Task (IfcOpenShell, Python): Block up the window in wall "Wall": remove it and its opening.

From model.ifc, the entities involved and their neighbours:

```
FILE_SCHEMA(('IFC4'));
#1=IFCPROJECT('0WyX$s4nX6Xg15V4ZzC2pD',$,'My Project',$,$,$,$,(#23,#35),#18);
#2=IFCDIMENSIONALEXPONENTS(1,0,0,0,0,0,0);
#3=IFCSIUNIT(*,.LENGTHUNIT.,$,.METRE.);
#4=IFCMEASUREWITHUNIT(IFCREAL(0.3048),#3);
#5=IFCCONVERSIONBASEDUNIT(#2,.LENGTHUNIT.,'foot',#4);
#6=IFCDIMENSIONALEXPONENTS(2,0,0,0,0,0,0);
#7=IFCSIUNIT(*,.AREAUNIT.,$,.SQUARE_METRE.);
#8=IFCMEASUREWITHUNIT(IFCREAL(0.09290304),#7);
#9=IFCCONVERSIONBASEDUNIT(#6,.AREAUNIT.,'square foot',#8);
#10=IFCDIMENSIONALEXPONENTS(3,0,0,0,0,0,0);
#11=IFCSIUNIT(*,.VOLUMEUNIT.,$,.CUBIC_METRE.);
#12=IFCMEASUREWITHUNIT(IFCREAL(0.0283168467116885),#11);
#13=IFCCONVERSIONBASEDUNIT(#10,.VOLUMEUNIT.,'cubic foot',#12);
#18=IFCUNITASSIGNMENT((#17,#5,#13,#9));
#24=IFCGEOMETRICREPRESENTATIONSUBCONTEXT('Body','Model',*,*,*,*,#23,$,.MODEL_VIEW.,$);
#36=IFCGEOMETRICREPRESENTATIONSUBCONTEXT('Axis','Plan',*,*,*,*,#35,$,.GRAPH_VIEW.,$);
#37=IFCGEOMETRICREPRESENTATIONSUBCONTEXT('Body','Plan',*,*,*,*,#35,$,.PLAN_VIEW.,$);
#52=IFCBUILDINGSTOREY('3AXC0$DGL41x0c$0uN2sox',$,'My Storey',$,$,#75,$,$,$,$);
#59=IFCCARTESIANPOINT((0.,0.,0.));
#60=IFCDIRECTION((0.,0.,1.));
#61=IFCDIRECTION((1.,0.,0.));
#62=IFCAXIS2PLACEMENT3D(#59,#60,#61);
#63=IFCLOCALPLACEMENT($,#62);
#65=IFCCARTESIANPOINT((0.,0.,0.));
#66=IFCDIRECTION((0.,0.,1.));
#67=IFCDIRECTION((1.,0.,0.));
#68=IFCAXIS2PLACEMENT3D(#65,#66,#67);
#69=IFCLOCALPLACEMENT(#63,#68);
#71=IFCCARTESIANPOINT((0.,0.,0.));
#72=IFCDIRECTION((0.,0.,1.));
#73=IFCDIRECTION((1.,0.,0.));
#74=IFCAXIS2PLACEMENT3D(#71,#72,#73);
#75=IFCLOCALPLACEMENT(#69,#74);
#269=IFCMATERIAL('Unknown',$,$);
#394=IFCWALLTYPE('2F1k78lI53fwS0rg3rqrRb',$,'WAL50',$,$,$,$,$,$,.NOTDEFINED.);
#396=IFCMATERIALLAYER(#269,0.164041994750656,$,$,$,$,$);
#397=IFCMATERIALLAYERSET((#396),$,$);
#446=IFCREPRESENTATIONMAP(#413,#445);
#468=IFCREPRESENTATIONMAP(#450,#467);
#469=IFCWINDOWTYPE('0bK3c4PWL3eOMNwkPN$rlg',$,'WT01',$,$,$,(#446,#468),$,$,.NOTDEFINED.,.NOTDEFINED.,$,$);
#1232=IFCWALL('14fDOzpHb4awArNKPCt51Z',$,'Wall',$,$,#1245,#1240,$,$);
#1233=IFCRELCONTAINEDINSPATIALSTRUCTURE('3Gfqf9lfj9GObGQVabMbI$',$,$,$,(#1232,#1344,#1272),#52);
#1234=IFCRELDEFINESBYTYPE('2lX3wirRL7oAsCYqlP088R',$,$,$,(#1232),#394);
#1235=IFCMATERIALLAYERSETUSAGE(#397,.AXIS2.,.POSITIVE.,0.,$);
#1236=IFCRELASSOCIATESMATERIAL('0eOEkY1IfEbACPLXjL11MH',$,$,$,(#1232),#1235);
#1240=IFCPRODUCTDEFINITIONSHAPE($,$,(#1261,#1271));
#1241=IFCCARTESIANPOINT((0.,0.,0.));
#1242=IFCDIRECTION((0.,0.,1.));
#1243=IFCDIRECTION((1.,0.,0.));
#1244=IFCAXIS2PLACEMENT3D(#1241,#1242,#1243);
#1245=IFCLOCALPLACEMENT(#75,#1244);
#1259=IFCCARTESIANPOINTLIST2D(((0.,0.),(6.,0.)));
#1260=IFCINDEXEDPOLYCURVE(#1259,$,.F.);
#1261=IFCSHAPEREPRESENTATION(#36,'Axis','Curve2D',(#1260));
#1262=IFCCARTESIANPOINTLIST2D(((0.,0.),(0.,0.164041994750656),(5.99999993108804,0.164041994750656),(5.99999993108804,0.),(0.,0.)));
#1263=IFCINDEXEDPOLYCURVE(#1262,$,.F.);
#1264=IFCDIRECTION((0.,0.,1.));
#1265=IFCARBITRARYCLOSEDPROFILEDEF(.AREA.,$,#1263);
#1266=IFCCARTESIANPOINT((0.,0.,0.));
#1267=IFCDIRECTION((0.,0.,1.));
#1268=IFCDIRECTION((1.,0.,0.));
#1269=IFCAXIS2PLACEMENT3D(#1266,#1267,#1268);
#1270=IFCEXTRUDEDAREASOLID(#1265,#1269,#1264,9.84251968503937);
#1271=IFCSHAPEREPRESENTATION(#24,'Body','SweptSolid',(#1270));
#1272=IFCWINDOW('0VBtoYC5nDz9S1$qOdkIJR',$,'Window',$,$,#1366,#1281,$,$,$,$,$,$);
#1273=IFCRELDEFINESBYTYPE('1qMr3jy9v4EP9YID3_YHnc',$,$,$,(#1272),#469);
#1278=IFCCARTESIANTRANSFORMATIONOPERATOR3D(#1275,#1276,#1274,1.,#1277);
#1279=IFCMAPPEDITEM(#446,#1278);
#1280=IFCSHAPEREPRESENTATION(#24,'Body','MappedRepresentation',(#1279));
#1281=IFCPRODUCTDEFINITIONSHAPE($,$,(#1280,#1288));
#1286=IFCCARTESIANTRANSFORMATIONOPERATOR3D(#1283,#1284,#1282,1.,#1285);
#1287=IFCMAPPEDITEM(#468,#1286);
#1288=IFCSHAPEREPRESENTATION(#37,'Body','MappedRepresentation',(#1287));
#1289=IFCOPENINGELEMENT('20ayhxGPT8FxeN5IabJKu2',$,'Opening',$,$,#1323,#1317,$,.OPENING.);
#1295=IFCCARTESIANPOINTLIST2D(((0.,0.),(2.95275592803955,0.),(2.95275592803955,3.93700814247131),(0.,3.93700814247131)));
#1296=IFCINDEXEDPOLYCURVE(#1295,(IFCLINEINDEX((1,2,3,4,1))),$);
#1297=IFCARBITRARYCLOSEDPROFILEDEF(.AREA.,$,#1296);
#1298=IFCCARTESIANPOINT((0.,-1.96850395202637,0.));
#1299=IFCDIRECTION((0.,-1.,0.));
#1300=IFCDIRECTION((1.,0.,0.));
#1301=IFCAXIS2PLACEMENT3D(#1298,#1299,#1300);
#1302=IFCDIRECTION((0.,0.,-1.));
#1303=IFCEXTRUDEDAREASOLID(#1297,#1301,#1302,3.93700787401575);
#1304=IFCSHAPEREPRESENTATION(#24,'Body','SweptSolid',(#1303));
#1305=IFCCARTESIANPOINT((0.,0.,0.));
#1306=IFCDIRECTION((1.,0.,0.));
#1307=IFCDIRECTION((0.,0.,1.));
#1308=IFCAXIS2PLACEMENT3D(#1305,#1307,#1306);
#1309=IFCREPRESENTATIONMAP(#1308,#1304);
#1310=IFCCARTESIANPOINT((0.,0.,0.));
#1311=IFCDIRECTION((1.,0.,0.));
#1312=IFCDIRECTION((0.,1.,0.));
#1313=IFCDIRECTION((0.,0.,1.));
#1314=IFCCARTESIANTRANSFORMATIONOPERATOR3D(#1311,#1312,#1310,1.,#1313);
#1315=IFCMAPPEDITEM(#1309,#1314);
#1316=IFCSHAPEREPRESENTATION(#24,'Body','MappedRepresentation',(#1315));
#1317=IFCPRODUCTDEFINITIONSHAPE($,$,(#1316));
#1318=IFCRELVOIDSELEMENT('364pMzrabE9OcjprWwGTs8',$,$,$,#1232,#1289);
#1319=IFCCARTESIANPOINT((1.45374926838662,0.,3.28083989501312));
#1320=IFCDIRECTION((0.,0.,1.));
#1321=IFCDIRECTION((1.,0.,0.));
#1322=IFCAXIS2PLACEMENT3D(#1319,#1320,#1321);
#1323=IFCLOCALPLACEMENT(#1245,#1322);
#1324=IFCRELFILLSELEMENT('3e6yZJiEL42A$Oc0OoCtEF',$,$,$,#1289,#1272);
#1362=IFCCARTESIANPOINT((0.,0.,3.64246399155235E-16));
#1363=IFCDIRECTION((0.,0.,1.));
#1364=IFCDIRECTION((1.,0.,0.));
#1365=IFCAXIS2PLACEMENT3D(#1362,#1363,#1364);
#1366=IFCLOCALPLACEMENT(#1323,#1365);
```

```python
import ifcopenshell
import ifcopenshell.api.feature
import ifcopenshell.api.root
import ifcopenshell.geom
import ifcopenshell.util.shape

model = ifcopenshell.open("model.ifc")
settings = ifcopenshell.geom.settings()


def volume(element):
    """Net volume in cubic metres, openings subtracted."""
    shape = ifcopenshell.geom.create_shape(settings, element)
    return ifcopenshell.util.shape.get_volume(shape.geometry)


window = model.by_guid("0VBtoYC5nDz9S1$qOdkIJR")
opening = window.FillsVoids[0].RelatingOpeningElement
wall = opening.VoidsElements[0].RelatingBuildingElement
before = volume(wall)

ifcopenshell.api.root.remove_product(model, product=window)
ifcopenshell.api.feature.remove_feature(model, feature=opening)

after = volume(wall)

print(f"wall volume {before:.3f} -> {after:.3f} m3")

model.write("model_rev.ifc")
```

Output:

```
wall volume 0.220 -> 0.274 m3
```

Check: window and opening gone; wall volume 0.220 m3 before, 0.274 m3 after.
